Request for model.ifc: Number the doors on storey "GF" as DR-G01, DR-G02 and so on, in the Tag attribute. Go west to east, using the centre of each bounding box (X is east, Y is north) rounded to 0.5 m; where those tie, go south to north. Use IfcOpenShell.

First a look at what the model holds.

```python
import ifcopenshell
import ifcopenshell.util.element
import ifcopenshell.util.placement

model = ifcopenshell.open("model.ifc")
print(model.schema)
storey = next(s for s in model.by_type("IfcBuildingStorey") if s.Name == "GF")
doors = [e for e in ifcopenshell.util.element.get_decomposition(storey) if e.is_a("IfcDoor")]
for e in sorted(doors, key=lambda e: e.id()):
    origin = ifcopenshell.util.placement.get_local_placement(e.ObjectPlacement)[:3, 3]
    print(e.id(), e.Tag, e.Name, origin.round(2) + 0.0, sep=" | ")
```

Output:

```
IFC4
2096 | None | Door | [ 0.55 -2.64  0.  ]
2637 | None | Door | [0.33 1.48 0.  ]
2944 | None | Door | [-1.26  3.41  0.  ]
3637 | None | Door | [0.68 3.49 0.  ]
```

```python
import ifcopenshell
import ifcopenshell.geom
import ifcopenshell.util.element
import ifcopenshell.util.shape

model = ifcopenshell.open("model.ifc")
settings = ifcopenshell.geom.settings()
settings.set("use-world-coords", True)


def centre(element):
    shape = ifcopenshell.geom.create_shape(settings, element)
    return ifcopenshell.util.shape.get_bbox_centroid(shape.geometry)


storey = next(s for s in model.by_type("IfcBuildingStorey") if s.Name == "GF")
doors = [e for e in ifcopenshell.util.element.get_decomposition(storey) if e.is_a("IfcDoor")]

# Insertion points can sit at a corner or the storey origin, so sort by the geometry (in metres).
centres = {e: centre(e) for e in doors}
doors.sort(key=lambda e: (round(centres[e][0] / 0.5), centres[e][1]))

for i, e in enumerate(doors, start=1):
    number = f"DR-G{i:02d}"
    e.Tag = number
    print(e.id(), number)

model.write("model-out.ifc")
```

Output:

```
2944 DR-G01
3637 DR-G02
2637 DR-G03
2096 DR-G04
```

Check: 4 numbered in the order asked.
